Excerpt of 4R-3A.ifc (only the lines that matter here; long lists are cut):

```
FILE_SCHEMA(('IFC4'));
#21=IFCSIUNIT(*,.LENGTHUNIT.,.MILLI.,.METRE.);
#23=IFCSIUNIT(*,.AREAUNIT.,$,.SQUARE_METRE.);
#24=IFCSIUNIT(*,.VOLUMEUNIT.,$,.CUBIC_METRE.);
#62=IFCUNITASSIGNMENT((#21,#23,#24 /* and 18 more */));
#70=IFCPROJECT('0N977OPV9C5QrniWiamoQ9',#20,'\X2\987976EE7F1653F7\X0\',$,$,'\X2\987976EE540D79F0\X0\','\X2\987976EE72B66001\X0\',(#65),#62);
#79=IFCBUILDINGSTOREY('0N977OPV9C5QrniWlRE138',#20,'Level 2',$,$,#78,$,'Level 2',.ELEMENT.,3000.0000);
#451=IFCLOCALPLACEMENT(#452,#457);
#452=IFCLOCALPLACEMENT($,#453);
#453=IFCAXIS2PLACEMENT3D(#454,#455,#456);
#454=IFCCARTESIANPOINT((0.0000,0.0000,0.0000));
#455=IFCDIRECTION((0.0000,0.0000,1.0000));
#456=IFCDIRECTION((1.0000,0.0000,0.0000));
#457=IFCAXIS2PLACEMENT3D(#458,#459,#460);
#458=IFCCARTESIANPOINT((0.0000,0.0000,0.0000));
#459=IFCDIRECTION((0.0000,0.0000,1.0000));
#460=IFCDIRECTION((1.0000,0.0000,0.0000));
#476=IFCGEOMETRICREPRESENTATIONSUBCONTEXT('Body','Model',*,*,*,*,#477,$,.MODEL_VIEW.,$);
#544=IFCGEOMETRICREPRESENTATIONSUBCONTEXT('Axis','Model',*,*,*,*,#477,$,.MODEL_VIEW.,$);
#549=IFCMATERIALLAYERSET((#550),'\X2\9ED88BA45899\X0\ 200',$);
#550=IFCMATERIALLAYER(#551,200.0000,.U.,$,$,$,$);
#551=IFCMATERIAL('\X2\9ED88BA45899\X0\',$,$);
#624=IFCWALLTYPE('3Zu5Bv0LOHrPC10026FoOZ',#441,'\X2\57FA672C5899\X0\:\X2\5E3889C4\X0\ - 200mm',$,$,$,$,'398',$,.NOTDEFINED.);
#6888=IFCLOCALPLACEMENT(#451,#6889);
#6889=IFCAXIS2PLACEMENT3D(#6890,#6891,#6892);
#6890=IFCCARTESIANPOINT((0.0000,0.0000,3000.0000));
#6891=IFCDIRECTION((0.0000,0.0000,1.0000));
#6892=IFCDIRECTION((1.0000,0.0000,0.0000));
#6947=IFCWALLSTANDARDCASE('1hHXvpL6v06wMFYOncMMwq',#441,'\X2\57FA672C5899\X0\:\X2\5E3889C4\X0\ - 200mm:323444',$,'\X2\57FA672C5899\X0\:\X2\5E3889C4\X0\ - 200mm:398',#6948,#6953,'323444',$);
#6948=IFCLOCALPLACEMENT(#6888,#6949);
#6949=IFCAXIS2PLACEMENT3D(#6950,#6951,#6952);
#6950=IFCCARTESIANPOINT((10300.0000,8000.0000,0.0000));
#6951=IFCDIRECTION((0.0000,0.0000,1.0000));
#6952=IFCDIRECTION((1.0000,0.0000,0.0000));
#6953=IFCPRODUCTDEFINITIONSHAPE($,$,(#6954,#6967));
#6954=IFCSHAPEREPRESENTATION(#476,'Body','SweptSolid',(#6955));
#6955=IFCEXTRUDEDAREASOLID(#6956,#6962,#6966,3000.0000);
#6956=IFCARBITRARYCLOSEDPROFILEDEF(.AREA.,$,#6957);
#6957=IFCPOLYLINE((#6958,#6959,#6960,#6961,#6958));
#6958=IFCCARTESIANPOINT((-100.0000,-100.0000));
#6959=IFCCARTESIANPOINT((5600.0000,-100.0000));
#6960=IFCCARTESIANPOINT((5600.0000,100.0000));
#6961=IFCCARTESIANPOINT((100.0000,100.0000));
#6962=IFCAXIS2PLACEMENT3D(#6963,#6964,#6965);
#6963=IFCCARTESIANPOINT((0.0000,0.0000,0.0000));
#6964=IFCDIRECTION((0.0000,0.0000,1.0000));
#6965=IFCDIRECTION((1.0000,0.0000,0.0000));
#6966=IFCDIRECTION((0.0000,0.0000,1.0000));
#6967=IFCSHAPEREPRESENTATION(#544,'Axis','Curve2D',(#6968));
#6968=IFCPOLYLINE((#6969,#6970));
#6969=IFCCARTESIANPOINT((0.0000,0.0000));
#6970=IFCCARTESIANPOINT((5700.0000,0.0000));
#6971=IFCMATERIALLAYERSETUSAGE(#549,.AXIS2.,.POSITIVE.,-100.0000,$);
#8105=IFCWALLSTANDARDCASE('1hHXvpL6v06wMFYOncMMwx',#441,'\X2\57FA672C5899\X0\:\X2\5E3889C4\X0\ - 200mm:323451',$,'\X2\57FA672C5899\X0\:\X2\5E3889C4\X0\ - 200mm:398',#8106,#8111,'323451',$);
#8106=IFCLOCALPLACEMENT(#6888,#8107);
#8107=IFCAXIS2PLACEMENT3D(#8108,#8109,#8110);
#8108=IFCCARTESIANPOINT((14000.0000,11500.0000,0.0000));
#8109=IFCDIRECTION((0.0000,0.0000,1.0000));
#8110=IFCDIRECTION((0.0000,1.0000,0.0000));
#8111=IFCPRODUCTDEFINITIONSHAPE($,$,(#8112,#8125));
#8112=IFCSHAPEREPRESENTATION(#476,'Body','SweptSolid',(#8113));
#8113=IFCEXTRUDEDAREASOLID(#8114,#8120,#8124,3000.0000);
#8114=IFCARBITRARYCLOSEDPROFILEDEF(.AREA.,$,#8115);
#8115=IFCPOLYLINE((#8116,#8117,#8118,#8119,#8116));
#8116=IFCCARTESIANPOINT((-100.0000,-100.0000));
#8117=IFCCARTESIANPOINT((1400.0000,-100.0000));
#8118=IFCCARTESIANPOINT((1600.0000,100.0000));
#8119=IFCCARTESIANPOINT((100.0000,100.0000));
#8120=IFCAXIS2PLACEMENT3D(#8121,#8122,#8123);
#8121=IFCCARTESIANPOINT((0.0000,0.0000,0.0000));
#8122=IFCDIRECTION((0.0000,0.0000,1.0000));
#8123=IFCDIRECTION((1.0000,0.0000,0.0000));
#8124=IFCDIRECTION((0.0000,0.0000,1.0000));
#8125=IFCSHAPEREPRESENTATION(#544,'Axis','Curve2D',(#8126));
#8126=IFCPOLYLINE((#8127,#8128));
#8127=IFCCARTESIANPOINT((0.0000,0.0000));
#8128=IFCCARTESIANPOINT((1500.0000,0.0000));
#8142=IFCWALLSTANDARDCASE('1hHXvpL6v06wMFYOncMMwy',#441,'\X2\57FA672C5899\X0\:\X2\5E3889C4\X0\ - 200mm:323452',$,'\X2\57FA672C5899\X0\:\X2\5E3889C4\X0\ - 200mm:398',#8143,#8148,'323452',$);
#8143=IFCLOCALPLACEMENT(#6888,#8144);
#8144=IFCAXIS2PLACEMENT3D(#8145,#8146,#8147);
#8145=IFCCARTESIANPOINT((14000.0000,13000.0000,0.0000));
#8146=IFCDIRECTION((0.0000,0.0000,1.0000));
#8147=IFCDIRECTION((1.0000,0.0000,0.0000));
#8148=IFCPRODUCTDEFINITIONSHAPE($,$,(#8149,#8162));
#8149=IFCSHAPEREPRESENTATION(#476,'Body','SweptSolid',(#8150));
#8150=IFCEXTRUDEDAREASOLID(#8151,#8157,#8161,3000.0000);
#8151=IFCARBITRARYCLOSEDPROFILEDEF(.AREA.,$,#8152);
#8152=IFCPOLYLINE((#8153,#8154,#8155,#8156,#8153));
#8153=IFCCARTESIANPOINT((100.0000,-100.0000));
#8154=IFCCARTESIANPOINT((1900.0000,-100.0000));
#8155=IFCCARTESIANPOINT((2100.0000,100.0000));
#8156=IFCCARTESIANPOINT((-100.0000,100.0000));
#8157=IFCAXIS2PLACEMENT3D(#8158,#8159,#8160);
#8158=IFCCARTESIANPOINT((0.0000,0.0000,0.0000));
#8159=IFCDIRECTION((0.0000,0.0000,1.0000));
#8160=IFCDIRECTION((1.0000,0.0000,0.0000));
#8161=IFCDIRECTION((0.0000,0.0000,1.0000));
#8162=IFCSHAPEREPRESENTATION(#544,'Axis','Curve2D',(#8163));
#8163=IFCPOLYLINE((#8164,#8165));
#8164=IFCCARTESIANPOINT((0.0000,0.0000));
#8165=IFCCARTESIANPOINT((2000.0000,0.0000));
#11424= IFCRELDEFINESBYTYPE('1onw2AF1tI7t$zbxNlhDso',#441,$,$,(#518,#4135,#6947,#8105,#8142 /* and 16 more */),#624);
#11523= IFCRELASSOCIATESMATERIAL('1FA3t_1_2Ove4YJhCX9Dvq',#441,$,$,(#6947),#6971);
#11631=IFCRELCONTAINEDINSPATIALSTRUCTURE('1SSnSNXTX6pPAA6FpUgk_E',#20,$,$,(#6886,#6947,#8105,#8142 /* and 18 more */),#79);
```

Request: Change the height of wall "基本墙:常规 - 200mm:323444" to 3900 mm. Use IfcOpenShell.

```python
import ifcopenshell
import ifcopenshell.geom
import ifcopenshell.util.representation
import ifcopenshell.util.shape
import ifcopenshell.util.unit

model = ifcopenshell.open("4R-3A.ifc")
unit_scale = ifcopenshell.util.unit.calculate_unit_scale(model)
settings = ifcopenshell.geom.settings()


def volume(element):
    """Net volume in cubic metres, openings subtracted."""
    shape = ifcopenshell.geom.create_shape(settings, element)
    return ifcopenshell.util.shape.get_volume(shape.geometry)


wall = model.by_guid("1hHXvpL6v06wMFYOncMMwq")
before = volume(wall)

body = ifcopenshell.util.representation.get_representation(wall, "Model", "Body")
solid = body.Items[0]
old_height = solid.Depth
solid.Depth = 3.9 / unit_scale
after = volume(wall)

print(f"height {old_height:g} -> {solid.Depth:g}, volume {before:.3f} -> {after:.3f} m3")

model.write("4R-3A_v2.ifc")
```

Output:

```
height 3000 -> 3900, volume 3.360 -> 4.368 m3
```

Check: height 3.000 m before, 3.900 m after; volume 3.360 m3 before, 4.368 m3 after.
